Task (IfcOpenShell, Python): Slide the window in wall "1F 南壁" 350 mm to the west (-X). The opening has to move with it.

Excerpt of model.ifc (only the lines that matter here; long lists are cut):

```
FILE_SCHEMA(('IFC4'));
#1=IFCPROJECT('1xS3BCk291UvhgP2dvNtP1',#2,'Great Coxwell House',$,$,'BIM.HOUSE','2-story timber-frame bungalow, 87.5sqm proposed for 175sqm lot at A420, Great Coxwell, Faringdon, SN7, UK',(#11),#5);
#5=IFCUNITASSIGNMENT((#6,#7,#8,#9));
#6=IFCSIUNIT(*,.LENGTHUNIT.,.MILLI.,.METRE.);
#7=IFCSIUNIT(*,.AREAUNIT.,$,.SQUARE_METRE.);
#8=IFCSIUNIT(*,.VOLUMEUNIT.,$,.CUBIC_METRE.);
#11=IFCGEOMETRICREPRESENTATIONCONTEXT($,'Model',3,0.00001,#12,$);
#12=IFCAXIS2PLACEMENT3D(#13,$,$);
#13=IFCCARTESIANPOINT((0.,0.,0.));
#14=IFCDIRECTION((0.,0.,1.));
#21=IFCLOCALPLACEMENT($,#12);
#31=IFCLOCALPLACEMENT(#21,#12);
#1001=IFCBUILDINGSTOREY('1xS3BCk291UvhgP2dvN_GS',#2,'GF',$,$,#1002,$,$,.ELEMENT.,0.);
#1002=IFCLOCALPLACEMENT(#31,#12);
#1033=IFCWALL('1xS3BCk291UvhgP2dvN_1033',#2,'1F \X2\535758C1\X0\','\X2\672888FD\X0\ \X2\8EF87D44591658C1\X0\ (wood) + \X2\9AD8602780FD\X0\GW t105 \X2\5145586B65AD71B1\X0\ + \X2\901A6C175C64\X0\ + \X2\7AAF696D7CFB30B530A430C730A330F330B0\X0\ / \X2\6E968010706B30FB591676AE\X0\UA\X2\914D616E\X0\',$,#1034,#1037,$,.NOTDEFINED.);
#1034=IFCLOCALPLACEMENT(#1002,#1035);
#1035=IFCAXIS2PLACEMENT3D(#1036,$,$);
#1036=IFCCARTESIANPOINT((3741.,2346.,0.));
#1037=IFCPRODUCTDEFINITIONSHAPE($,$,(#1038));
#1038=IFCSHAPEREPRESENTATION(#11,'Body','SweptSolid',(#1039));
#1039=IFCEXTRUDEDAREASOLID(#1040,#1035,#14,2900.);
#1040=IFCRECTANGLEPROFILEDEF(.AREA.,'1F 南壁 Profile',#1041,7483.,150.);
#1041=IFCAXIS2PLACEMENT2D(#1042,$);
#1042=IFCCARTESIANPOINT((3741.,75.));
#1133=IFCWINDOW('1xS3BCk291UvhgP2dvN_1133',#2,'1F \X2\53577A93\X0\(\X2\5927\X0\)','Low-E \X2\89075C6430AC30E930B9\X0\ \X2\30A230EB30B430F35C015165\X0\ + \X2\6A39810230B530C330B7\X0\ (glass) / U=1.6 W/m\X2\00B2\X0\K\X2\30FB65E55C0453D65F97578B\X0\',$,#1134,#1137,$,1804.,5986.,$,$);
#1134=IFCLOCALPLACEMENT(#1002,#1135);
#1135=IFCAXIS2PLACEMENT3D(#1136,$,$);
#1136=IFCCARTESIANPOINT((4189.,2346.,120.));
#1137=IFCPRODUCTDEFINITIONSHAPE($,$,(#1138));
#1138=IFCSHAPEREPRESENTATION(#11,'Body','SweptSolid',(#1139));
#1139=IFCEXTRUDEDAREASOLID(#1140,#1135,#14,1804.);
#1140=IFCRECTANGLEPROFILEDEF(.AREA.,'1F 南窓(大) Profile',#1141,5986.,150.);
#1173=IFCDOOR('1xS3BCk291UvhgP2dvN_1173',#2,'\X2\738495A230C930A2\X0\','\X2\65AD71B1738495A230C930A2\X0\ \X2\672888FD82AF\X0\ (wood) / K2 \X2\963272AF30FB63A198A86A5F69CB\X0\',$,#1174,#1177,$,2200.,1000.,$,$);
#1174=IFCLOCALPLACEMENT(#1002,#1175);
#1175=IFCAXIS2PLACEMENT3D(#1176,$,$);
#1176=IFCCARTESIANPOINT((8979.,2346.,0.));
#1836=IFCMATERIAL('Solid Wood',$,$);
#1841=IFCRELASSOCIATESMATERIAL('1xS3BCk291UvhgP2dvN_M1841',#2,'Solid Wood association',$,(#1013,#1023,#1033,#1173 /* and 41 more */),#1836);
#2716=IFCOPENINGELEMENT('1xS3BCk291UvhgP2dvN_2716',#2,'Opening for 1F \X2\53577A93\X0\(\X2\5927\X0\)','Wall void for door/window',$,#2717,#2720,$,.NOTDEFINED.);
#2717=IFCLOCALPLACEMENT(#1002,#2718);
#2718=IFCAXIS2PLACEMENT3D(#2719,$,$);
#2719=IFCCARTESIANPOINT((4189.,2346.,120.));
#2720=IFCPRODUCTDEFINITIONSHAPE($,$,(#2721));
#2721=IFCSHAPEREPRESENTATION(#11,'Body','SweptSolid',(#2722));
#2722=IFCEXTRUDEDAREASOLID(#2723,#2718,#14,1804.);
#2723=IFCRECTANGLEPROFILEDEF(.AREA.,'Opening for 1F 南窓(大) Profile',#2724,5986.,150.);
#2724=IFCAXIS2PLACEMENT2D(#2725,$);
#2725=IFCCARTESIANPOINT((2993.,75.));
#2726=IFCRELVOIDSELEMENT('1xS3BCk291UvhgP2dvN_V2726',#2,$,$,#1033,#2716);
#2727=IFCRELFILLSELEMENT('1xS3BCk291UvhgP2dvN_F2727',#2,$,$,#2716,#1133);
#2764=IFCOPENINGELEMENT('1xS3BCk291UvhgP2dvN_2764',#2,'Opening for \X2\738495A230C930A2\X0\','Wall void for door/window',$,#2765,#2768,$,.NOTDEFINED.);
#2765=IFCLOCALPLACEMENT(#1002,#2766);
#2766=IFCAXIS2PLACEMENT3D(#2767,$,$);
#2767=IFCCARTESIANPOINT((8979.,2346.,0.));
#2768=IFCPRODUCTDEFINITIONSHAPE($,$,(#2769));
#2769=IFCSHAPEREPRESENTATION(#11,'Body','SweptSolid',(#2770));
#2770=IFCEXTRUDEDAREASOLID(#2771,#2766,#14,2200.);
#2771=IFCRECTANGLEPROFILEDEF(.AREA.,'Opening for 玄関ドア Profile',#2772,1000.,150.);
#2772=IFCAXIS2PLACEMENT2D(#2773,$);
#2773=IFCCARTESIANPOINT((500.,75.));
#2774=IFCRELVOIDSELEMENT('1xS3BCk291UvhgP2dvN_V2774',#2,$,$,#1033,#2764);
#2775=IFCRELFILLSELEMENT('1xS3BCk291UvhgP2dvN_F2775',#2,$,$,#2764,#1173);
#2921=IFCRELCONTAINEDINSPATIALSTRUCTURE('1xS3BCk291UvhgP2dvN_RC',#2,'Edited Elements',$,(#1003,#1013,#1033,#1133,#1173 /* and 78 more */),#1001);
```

```python
import ifcopenshell
import ifcopenshell.api.geometry
import ifcopenshell.util.placement

model = ifcopenshell.open("model.ifc")

window = model.by_id(1133)
opening = window.FillsVoids[0].RelatingOpeningElement
wall = opening.VoidsElements[0].RelatingBuildingElement

wall_matrix = ifcopenshell.util.placement.get_local_placement(wall.ObjectPlacement)
shift = wall_matrix[:3, 0] * -350.0
before = ifcopenshell.util.placement.get_local_placement(window.ObjectPlacement)[:3, 3].copy()

# The window is not placed relative to its opening, so move both.
for product in (opening, window):
    matrix = ifcopenshell.util.placement.get_local_placement(product.ObjectPlacement)
    matrix[:3, 3] += shift
    ifcopenshell.api.geometry.edit_object_placement(model, product=product, matrix=matrix, is_si=False)

after = ifcopenshell.util.placement.get_local_placement(window.ObjectPlacement)[:3, 3]
print("window moved by", (after - before).round(3) + 0.0)

model.write("model_edited.ifc")
```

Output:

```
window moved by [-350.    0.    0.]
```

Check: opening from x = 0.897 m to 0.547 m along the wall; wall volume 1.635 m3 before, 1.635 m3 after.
